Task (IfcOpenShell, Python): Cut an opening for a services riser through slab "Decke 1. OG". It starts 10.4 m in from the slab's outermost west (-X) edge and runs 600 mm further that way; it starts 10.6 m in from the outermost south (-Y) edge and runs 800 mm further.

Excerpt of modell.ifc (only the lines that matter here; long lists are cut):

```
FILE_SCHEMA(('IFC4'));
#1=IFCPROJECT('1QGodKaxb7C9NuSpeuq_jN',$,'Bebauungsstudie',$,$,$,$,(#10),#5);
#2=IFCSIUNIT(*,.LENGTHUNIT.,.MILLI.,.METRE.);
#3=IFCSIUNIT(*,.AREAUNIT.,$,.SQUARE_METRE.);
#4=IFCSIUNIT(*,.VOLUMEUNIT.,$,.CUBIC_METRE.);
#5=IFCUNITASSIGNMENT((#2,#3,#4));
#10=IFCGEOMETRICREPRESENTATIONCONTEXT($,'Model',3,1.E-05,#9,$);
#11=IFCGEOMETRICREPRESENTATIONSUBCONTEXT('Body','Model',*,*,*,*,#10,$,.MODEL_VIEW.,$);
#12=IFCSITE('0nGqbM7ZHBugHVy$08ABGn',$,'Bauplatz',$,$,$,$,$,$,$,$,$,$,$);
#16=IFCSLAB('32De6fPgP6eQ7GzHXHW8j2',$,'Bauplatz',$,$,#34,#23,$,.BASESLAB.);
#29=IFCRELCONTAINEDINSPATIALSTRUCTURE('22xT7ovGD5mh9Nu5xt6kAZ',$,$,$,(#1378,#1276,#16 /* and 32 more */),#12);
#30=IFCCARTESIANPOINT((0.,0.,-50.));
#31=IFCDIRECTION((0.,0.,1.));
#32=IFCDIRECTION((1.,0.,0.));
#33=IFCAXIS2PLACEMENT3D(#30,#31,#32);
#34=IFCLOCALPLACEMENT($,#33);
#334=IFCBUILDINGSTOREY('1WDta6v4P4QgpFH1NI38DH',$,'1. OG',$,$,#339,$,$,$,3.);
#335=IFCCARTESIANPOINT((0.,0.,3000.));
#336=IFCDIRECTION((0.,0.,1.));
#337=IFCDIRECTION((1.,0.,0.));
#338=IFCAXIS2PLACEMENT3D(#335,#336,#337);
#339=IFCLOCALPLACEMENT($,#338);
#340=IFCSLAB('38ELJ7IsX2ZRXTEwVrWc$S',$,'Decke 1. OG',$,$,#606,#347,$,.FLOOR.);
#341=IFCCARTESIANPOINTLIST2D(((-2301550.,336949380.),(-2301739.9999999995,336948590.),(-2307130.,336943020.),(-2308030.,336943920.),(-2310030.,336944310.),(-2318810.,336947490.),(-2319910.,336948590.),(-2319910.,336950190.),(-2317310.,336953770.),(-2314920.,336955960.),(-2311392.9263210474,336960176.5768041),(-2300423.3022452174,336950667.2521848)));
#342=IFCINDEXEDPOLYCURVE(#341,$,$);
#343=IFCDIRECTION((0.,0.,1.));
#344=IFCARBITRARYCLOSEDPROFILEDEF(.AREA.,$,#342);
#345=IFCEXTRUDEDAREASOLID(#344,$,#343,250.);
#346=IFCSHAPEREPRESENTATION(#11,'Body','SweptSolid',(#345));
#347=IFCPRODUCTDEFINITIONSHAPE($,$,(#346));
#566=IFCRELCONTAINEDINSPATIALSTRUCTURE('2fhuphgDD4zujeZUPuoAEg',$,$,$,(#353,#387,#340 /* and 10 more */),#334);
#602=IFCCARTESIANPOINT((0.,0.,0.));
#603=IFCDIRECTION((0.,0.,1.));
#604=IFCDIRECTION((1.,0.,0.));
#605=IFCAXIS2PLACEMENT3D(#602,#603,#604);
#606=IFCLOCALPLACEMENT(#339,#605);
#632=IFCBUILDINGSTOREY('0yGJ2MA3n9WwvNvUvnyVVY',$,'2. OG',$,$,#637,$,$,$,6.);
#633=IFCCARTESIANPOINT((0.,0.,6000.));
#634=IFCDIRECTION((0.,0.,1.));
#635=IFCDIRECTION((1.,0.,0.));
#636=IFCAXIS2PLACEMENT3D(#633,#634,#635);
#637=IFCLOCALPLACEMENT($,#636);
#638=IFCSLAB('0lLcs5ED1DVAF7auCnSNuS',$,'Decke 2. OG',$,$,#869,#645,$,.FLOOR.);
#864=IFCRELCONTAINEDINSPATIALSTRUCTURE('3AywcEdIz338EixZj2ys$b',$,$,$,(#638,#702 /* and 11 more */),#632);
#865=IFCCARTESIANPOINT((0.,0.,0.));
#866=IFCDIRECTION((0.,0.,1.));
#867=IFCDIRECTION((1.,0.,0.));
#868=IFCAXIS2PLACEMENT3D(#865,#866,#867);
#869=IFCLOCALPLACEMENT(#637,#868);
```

```python
import numpy as np
import ifcopenshell
import ifcopenshell.api.feature
import ifcopenshell.api.geometry
import ifcopenshell.api.root
import ifcopenshell.geom
import ifcopenshell.util.placement
import ifcopenshell.util.representation
import ifcopenshell.util.shape
import ifcopenshell.util.unit

model = ifcopenshell.open("modell.ifc")
unit_scale = ifcopenshell.util.unit.calculate_unit_scale(model)
settings = ifcopenshell.geom.settings()


def volume(element):
    """Net volume in cubic metres, openings subtracted."""
    shape = ifcopenshell.geom.create_shape(settings, element)
    return ifcopenshell.util.shape.get_volume(shape.geometry)


slab = model.by_id(340)
before = volume(slab)

# Extent in the slab's own axes, in metres. The edges named are its -X and -Y sides.
slab_shape = ifcopenshell.geom.create_shape(settings, slab)
vertices = ifcopenshell.util.shape.get_vertices(slab_shape.geometry)
x_min, y_min, bottom = vertices.min(axis=0)
top = vertices[:, 2].max()

opening = ifcopenshell.api.root.create_entity(model, ifc_class="IfcOpeningElement", name="Services riser opening", predefined_type="OPENING")
context = ifcopenshell.util.representation.get_context(model, "Model", "Body", "MODEL_VIEW")
width, depth = 0.6, 0.8
outline = [(0.0, 0.0), (width, 0.0), (width, depth), (0.0, depth), (0.0, 0.0)]
# Overshoot both faces by 50 mm so the cut is clean.
shape = ifcopenshell.api.geometry.add_slab_representation(
    model, context=context, depth=top - bottom + 0.1, polyline=outline
)
ifcopenshell.api.geometry.assign_representation(model, product=opening, representation=shape)

matrix = ifcopenshell.util.placement.get_local_placement(slab.ObjectPlacement)
matrix[:, 3] = matrix @ np.append(np.array([x_min + 10.4, y_min + 10.6, bottom - 0.05]) / unit_scale, 1.0)
ifcopenshell.api.geometry.edit_object_placement(model, product=opening, matrix=matrix, is_si=False)
ifcopenshell.api.feature.add_feature(model, feature=opening, element=slab)

after = volume(slab)

print(f"slab volume {before:.3f} -> {after:.3f} m3")

model.write("modell_edited.ifc")
```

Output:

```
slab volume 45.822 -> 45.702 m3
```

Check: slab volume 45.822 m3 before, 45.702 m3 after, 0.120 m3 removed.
